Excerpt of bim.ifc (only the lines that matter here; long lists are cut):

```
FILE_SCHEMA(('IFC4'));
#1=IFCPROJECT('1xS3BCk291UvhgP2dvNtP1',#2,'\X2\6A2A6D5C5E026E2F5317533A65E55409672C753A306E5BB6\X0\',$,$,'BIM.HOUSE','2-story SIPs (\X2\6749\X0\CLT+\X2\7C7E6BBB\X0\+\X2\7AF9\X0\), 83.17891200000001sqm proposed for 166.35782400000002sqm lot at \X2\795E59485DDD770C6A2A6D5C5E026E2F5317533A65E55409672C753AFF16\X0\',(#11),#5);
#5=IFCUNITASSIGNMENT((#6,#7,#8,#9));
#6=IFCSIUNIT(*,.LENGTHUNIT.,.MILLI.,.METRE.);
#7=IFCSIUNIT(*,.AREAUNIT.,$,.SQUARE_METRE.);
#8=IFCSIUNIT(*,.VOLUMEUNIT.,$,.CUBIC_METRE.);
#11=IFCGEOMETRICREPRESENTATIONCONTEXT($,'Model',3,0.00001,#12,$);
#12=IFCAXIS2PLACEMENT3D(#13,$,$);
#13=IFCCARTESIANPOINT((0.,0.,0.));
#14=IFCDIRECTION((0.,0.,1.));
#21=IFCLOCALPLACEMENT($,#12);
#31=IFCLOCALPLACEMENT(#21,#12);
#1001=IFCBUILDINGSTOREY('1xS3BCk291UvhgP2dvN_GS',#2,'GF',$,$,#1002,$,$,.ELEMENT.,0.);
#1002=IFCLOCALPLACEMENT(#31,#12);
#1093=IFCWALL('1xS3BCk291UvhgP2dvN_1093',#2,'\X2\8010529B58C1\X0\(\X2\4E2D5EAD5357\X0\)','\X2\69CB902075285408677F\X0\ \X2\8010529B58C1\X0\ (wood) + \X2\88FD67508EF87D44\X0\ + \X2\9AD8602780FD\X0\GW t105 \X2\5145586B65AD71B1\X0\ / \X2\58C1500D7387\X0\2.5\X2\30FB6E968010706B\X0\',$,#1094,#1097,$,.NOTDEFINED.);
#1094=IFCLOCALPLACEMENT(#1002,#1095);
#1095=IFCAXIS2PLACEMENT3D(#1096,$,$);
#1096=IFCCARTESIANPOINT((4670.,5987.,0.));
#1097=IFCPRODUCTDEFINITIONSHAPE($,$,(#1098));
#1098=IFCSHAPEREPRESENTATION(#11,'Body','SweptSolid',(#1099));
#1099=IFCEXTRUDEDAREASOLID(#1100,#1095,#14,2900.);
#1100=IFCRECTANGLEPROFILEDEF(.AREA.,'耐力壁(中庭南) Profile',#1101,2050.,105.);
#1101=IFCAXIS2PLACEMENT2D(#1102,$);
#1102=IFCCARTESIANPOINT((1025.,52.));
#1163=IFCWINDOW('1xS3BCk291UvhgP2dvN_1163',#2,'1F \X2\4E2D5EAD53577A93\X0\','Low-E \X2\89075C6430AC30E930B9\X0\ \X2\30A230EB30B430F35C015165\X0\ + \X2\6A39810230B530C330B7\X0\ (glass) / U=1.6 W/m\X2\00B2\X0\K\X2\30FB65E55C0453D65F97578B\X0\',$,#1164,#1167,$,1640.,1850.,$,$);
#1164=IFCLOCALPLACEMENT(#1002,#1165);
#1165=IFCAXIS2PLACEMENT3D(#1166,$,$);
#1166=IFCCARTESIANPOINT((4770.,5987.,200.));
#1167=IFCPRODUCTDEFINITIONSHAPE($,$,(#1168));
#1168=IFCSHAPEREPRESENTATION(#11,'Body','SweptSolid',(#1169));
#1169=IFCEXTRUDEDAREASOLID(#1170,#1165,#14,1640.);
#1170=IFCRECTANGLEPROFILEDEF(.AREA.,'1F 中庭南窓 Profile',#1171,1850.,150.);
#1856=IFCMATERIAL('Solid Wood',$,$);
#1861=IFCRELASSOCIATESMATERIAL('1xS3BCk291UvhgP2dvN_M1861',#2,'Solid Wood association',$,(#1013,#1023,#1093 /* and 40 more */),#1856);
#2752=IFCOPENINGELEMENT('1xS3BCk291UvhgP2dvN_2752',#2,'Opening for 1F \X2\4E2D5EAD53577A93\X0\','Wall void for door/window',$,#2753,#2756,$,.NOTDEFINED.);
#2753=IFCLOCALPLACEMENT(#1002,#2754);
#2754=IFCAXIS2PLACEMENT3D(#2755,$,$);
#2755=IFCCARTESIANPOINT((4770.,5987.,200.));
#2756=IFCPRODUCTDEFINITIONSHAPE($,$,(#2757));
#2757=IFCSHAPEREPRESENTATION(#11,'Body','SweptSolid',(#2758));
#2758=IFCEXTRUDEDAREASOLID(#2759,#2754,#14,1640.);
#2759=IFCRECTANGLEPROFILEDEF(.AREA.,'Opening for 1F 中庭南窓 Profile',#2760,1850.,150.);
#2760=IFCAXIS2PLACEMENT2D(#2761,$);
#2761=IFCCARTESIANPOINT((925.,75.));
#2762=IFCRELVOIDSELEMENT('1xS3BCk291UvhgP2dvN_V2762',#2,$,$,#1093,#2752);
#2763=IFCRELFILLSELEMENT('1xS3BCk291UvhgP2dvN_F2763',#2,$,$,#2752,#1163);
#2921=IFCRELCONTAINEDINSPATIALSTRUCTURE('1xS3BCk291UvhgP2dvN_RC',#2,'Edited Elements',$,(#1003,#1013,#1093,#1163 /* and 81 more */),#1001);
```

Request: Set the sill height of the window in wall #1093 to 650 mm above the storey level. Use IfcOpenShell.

```python
import numpy as np
import ifcopenshell
import ifcopenshell.api.geometry
import ifcopenshell.geom
import ifcopenshell.util.element
import ifcopenshell.util.placement
import ifcopenshell.util.shape
import ifcopenshell.util.unit

model = ifcopenshell.open("bim.ifc")
unit_scale = ifcopenshell.util.unit.calculate_unit_scale(model)

window = model.by_guid("1xS3BCk291UvhgP2dvN_1163")
opening = window.FillsVoids[0].RelatingOpeningElement
storey = ifcopenshell.util.element.get_container(window, ifc_class="IfcBuildingStorey")
level = ifcopenshell.util.placement.get_local_placement(storey.ObjectPlacement)[2, 3]

# The opening's origin need not be at the sill, so measure its lowest point.
shape = ifcopenshell.geom.create_shape(ifcopenshell.geom.settings(), opening)
bottom = ifcopenshell.util.shape.get_shape_bottom_elevation(shape, shape.geometry) / unit_scale
dz = level + 0.65 / unit_scale - bottom

shift = np.array([0.0, 0.0, dz])
# The window is not placed relative to its opening, so move both.
for product in (opening, window):
    matrix = ifcopenshell.util.placement.get_local_placement(product.ObjectPlacement)
    matrix[:3, 3] += shift
    ifcopenshell.api.geometry.edit_object_placement(model, product=product, matrix=matrix, is_si=False)

print(f"moved by {dz * unit_scale:+.3f} m")

model.write("bim_v2.ifc")
```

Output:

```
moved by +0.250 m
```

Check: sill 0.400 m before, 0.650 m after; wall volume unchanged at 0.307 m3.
